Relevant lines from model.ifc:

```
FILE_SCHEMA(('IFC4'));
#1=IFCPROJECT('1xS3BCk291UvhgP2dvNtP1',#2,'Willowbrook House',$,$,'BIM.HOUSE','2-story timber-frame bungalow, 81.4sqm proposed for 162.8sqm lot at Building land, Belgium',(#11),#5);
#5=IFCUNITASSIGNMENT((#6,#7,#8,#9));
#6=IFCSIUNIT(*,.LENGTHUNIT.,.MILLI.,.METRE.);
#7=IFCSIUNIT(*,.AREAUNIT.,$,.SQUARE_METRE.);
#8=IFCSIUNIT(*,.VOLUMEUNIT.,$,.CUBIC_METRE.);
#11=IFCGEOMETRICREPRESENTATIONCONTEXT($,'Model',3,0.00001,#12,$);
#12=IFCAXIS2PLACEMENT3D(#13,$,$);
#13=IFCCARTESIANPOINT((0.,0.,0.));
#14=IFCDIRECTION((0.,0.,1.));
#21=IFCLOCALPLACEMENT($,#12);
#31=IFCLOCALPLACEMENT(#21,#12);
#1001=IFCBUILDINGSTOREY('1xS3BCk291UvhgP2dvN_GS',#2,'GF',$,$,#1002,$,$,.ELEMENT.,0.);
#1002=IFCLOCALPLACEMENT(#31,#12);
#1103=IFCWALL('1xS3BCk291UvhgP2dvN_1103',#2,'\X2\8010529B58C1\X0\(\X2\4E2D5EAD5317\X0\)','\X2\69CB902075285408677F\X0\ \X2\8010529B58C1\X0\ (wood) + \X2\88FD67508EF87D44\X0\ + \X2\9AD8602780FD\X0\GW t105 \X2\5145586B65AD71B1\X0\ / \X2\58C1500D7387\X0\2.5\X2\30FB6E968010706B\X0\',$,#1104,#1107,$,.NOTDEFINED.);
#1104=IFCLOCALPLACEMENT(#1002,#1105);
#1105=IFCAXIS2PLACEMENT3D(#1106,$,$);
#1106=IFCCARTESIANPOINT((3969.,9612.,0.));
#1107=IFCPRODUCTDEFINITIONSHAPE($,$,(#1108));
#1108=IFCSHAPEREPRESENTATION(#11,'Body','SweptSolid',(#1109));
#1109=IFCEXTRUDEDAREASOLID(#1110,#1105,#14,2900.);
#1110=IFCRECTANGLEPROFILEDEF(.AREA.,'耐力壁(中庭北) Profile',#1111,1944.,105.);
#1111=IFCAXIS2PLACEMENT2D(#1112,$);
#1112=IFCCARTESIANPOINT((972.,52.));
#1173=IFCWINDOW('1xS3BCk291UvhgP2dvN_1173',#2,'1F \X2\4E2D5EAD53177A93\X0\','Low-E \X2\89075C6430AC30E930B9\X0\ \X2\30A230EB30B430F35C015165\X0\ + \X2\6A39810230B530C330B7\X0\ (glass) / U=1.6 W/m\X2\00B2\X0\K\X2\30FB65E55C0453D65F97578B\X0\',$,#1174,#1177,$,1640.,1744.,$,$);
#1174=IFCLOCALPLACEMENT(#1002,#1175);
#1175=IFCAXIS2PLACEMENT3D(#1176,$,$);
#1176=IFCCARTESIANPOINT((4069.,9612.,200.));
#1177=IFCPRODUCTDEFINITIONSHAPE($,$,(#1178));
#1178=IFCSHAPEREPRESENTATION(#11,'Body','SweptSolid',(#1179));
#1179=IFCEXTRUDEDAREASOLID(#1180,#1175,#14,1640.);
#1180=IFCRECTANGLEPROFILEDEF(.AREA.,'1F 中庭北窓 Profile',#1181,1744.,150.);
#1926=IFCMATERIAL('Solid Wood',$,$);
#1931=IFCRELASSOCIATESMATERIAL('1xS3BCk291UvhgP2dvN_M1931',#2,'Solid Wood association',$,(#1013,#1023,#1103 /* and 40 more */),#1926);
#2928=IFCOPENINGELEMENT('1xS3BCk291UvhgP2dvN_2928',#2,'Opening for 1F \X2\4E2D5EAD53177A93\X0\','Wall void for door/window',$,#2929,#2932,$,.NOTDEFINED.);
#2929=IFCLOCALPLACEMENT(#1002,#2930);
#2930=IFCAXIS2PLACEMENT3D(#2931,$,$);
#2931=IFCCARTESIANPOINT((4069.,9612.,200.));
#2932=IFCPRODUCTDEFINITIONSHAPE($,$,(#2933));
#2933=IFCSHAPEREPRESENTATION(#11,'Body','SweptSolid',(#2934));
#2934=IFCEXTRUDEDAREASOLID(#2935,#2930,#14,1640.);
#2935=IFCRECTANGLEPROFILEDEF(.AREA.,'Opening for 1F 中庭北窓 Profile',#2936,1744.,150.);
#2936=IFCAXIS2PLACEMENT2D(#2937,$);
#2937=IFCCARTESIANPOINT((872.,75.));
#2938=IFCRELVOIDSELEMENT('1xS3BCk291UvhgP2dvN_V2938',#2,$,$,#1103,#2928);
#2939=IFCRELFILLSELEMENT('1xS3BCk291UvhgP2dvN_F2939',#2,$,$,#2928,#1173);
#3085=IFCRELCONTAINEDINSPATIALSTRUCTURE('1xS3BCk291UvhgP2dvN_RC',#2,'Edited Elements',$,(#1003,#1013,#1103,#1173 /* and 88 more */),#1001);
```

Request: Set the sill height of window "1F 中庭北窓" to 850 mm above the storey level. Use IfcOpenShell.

```python
import numpy as np
import ifcopenshell
import ifcopenshell.api.geometry
import ifcopenshell.geom
import ifcopenshell.util.element
import ifcopenshell.util.placement
import ifcopenshell.util.shape
import ifcopenshell.util.unit

model = ifcopenshell.open("model.ifc")
unit_scale = ifcopenshell.util.unit.calculate_unit_scale(model)

window = model.by_id(1173)
opening = window.FillsVoids[0].RelatingOpeningElement
storey = ifcopenshell.util.element.get_container(window, ifc_class="IfcBuildingStorey")
level = ifcopenshell.util.placement.get_local_placement(storey.ObjectPlacement)[2, 3]

# The opening's origin need not be at the sill, so measure its lowest point.
shape = ifcopenshell.geom.create_shape(ifcopenshell.geom.settings(), opening)
bottom = ifcopenshell.util.shape.get_shape_bottom_elevation(shape, shape.geometry) / unit_scale
dz = level + 0.85 / unit_scale - bottom

shift = np.array([0.0, 0.0, dz])
# The window is not placed relative to its opening, so move both.
for product in (opening, window):
    matrix = ifcopenshell.util.placement.get_local_placement(product.ObjectPlacement)
    matrix[:3, 3] += shift
    ifcopenshell.api.geometry.edit_object_placement(model, product=product, matrix=matrix, is_si=False)

print(f"moved by {dz * unit_scale:+.3f} m")

model.write("model_updated.ifc")
```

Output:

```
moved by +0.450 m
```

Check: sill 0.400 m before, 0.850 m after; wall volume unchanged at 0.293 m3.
